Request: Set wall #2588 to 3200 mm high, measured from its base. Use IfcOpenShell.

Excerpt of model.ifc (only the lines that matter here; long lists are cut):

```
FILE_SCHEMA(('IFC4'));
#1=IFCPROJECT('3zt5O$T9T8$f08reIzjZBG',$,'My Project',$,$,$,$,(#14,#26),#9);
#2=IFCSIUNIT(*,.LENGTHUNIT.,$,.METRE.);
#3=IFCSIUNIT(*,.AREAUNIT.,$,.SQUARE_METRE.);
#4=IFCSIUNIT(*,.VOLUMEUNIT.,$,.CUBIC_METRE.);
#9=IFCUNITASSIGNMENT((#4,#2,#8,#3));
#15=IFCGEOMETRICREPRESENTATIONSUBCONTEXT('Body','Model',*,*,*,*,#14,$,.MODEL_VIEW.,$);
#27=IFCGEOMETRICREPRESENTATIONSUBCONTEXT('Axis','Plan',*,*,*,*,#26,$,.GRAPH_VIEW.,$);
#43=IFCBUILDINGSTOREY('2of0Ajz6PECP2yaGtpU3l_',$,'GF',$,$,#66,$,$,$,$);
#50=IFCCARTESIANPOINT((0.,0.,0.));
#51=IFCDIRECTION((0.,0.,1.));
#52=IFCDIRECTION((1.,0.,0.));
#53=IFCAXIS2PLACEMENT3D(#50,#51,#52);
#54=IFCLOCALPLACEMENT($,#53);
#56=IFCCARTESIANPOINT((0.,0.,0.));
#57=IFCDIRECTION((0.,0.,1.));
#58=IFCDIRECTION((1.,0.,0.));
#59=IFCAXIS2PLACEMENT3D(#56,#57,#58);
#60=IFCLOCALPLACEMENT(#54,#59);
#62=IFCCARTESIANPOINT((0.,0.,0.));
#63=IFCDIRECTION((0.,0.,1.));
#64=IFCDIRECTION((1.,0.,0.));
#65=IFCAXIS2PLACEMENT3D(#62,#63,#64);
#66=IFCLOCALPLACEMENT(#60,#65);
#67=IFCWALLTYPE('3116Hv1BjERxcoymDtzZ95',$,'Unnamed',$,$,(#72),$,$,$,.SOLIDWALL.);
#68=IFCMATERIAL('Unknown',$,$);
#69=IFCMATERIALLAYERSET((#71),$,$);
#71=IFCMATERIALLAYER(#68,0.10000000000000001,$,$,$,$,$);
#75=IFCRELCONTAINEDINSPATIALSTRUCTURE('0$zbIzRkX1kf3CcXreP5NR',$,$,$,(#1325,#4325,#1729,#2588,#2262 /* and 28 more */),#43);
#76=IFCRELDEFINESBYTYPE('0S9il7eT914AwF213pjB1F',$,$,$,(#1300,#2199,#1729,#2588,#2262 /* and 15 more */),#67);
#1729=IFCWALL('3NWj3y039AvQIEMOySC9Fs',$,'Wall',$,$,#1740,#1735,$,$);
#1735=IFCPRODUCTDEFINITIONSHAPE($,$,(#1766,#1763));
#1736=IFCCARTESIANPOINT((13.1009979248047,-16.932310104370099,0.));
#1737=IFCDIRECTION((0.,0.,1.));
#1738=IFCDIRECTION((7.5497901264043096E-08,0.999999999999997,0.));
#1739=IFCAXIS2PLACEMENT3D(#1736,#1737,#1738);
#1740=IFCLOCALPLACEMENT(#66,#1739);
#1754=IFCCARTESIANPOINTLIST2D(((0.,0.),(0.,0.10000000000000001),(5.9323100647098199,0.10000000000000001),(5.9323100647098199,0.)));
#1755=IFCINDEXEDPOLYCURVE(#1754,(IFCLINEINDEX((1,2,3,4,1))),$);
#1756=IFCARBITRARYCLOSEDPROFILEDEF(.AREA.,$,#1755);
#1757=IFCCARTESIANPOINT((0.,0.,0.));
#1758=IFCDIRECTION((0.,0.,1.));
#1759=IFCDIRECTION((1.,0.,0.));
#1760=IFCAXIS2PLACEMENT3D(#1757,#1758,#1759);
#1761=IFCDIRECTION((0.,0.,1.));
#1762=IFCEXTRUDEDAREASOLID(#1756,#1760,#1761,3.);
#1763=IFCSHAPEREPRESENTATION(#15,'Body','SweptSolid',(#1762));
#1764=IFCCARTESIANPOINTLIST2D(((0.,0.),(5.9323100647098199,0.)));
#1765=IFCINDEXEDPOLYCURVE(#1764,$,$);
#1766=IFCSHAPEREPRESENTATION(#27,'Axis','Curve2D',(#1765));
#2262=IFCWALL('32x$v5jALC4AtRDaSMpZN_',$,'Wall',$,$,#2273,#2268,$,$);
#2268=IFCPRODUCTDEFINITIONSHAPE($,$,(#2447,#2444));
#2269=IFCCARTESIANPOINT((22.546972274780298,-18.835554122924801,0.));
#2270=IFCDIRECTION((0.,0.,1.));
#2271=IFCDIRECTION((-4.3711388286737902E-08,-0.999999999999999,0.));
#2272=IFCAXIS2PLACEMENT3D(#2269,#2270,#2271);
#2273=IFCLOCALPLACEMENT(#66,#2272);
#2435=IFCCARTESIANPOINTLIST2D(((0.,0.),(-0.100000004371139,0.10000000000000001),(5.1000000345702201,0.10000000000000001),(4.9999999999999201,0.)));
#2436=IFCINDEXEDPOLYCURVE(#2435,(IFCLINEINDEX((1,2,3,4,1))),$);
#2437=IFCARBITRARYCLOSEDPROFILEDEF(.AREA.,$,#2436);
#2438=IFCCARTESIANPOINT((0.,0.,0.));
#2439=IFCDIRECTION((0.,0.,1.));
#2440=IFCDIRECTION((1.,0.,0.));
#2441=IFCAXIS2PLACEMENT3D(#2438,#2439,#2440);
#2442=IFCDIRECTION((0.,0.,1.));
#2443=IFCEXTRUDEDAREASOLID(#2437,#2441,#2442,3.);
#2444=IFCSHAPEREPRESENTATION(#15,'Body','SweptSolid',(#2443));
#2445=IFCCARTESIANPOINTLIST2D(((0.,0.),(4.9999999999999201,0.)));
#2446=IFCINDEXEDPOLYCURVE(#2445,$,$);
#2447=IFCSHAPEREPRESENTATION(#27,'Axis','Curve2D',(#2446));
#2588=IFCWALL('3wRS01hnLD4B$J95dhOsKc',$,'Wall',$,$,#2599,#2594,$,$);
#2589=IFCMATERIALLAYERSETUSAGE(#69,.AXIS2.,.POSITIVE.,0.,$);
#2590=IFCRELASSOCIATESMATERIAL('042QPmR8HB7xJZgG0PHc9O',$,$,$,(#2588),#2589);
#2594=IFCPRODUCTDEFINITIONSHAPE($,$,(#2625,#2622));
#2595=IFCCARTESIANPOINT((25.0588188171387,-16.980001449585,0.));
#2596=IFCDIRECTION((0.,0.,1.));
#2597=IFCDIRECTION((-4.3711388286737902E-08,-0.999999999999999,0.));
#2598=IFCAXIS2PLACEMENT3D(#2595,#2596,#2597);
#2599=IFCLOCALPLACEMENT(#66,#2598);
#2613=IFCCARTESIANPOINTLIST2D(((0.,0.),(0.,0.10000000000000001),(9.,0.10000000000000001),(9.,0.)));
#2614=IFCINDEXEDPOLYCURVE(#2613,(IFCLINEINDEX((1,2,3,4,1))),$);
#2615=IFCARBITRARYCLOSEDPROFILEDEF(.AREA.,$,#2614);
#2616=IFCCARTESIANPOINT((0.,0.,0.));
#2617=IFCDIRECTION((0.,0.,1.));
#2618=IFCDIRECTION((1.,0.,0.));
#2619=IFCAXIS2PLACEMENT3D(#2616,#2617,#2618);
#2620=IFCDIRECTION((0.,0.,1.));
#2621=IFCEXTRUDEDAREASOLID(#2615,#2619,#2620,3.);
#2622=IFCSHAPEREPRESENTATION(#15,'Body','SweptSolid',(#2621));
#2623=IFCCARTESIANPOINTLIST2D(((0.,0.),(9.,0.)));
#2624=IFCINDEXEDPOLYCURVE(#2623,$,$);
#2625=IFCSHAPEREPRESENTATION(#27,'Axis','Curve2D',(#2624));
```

```python
import ifcopenshell
import ifcopenshell.geom
import ifcopenshell.util.representation
import ifcopenshell.util.shape

model = ifcopenshell.open("model.ifc")
settings = ifcopenshell.geom.settings()


def volume(element):
    """Net volume in cubic metres, openings subtracted."""
    shape = ifcopenshell.geom.create_shape(settings, element)
    return ifcopenshell.util.shape.get_volume(shape.geometry)


wall = model.by_guid("3wRS01hnLD4B$J95dhOsKc")
before = volume(wall)

body = ifcopenshell.util.representation.get_representation(wall, "Model", "Body")
solid = body.Items[0]
old_height = solid.Depth
solid.Depth = 3.2
after = volume(wall)

print(f"height {old_height:g} -> {solid.Depth:g}, volume {before:.3f} -> {after:.3f} m3")

model.write("model-out.ifc")
```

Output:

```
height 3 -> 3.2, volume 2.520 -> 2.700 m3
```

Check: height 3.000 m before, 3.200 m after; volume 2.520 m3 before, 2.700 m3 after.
